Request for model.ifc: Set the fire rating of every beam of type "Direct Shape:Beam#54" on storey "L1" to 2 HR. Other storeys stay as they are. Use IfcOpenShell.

First a look at what the model holds.

```python
import ifcopenshell
import ifcopenshell.util.element

model = ifcopenshell.open("model.ifc")
print(model.schema)
storey = next(s for s in model.by_type("IfcBuildingStorey") if s.Name == "L1")
beams = [e for e in ifcopenshell.util.element.get_decomposition(storey) if e.is_a("IfcBeam")]
seen = {}
for e in beams:
    element_type = ifcopenshell.util.element.get_type(e)
    key = (element_type.Name if element_type != e and element_type else None, ifcopenshell.util.element.get_pset(e, "Pset_BeamCommon", "FireRating"))
    seen[key] = seen.get(key, 0) + 1
for (name, value), count in sorted(seen.items(), key=str):
    print(count, "x", name, "|", value)
```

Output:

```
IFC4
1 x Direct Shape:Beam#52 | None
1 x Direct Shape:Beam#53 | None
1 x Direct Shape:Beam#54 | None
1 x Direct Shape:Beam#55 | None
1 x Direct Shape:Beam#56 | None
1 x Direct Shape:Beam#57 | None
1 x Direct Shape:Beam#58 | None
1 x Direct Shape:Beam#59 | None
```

```python
import ifcopenshell
import ifcopenshell.api.pset
import ifcopenshell.util.element

model = ifcopenshell.open("model.ifc")

storey = next(s for s in model.by_type("IfcBuildingStorey") if s.Name == "L1")
beams = [e for e in ifcopenshell.util.element.get_decomposition(storey) if e.is_a("IfcBeam")]

count = 0
for e in beams:
    element_type = ifcopenshell.util.element.get_type(e)
    if element_type in (None, e) or element_type.Name != "Direct Shape:Beam#54":
        continue
    # add_pset returns the element's existing set when there is one.
    pset = ifcopenshell.api.pset.add_pset(model, product=e, name="Pset_BeamCommon")
    ifcopenshell.api.pset.edit_pset(model, pset=pset, properties={"FireRating": "2 HR"})
    count += 1

print(count, "beams updated")

model.write("model-out.ifc")
```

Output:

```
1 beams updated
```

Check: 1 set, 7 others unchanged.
